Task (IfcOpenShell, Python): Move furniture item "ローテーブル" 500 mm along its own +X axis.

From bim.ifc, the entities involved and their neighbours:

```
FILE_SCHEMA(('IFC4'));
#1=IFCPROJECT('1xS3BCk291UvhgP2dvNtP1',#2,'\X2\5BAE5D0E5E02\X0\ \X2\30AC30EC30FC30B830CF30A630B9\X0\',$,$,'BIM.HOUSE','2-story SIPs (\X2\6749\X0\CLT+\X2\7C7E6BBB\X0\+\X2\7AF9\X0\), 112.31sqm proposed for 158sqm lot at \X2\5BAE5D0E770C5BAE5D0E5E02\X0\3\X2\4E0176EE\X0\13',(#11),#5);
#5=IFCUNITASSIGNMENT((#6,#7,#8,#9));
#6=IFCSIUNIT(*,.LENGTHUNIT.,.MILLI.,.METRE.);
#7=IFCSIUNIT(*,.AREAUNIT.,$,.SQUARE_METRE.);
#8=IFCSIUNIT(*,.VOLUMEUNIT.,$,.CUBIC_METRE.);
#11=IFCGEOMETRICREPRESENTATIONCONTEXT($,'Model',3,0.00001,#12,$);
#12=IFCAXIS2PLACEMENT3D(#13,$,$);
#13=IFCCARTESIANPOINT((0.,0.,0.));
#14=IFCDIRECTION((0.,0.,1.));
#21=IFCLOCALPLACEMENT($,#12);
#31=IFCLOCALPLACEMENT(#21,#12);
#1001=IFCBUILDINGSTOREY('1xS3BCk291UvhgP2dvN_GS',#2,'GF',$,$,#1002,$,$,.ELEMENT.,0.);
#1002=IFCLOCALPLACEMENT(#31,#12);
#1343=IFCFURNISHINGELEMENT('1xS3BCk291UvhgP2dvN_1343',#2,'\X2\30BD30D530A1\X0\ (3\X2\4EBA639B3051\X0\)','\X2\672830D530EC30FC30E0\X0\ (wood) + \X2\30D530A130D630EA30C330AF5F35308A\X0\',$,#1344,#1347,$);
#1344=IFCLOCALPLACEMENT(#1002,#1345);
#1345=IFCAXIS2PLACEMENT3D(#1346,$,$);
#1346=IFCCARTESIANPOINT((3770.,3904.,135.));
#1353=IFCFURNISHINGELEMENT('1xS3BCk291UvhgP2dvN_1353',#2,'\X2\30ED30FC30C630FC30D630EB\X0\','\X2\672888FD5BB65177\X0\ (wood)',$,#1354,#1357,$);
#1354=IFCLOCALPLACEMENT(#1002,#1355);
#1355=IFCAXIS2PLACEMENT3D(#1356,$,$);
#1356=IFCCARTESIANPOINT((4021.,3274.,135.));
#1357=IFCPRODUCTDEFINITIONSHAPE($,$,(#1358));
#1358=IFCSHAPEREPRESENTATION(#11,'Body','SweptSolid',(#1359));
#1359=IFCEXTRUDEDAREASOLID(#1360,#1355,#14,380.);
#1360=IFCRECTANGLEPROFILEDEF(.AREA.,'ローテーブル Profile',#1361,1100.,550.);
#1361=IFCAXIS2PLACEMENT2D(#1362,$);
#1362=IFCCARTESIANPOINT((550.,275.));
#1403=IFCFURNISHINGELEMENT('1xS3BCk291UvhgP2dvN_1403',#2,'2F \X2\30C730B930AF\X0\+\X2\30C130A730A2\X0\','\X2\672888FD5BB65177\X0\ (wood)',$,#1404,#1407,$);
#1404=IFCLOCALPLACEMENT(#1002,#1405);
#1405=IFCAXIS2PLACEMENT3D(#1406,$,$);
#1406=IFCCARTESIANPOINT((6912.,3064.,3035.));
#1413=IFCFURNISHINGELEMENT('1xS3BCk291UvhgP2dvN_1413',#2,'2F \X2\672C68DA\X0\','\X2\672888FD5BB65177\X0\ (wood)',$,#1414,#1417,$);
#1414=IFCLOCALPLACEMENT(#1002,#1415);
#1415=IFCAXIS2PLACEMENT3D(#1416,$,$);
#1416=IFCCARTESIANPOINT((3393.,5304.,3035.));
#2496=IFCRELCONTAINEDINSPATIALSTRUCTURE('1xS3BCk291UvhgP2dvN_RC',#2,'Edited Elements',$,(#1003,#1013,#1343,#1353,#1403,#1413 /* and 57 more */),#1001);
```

```python
import ifcopenshell
import ifcopenshell.api.geometry
import ifcopenshell.util.placement

model = ifcopenshell.open("bim.ifc")

item = model.by_id(1353)
matrix = ifcopenshell.util.placement.get_local_placement(item.ObjectPlacement)
matrix[:3, 3] += matrix[:3, 0] * 500.0
ifcopenshell.api.geometry.edit_object_placement(model, product=item, matrix=matrix, is_si=False)

print(ifcopenshell.util.placement.get_local_placement(item.ObjectPlacement).round(3) + 0.0)

model.write("bim_updated.ifc")
```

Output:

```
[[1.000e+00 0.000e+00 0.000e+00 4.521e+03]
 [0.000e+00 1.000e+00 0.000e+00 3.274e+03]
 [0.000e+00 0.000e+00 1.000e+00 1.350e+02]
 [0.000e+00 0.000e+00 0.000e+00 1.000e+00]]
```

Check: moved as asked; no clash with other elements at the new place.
